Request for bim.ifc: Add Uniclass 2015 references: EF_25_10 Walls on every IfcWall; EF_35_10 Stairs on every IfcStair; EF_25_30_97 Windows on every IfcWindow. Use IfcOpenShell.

First a look at what the model holds.

```python
import ifcopenshell

model = ifcopenshell.open("bim.ifc")
print(model.schema)
print("classifications:", [c.Name for c in model.by_type("IfcClassification")])
for ifc_class in ("IfcDoor", "IfcRoof", "IfcStair", "IfcWall", "IfcWindow"):
    print(ifc_class, len(model.by_type(ifc_class)))
```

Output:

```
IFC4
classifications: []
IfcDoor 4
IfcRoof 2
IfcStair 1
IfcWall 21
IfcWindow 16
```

```python
import ifcopenshell
import ifcopenshell.api.classification

model = ifcopenshell.open("bim.ifc")

system = ifcopenshell.api.classification.add_classification(model, classification="Uniclass 2015")

codes = {
    "IfcWall": ("EF_25_10", "Walls"),
    "IfcStair": ("EF_35_10", "Stairs"),
    "IfcWindow": ("EF_25_30_97", "Windows"),
}
for ifc_class, (code, name) in codes.items():
    products = model.by_type(ifc_class)
    ifcopenshell.api.classification.add_reference(
        model, products=products, classification=system, identification=code, name=name
    )
    print(code, len(products))

model.write("bim_v2.ifc")
```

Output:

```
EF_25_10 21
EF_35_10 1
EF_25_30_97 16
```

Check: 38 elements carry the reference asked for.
